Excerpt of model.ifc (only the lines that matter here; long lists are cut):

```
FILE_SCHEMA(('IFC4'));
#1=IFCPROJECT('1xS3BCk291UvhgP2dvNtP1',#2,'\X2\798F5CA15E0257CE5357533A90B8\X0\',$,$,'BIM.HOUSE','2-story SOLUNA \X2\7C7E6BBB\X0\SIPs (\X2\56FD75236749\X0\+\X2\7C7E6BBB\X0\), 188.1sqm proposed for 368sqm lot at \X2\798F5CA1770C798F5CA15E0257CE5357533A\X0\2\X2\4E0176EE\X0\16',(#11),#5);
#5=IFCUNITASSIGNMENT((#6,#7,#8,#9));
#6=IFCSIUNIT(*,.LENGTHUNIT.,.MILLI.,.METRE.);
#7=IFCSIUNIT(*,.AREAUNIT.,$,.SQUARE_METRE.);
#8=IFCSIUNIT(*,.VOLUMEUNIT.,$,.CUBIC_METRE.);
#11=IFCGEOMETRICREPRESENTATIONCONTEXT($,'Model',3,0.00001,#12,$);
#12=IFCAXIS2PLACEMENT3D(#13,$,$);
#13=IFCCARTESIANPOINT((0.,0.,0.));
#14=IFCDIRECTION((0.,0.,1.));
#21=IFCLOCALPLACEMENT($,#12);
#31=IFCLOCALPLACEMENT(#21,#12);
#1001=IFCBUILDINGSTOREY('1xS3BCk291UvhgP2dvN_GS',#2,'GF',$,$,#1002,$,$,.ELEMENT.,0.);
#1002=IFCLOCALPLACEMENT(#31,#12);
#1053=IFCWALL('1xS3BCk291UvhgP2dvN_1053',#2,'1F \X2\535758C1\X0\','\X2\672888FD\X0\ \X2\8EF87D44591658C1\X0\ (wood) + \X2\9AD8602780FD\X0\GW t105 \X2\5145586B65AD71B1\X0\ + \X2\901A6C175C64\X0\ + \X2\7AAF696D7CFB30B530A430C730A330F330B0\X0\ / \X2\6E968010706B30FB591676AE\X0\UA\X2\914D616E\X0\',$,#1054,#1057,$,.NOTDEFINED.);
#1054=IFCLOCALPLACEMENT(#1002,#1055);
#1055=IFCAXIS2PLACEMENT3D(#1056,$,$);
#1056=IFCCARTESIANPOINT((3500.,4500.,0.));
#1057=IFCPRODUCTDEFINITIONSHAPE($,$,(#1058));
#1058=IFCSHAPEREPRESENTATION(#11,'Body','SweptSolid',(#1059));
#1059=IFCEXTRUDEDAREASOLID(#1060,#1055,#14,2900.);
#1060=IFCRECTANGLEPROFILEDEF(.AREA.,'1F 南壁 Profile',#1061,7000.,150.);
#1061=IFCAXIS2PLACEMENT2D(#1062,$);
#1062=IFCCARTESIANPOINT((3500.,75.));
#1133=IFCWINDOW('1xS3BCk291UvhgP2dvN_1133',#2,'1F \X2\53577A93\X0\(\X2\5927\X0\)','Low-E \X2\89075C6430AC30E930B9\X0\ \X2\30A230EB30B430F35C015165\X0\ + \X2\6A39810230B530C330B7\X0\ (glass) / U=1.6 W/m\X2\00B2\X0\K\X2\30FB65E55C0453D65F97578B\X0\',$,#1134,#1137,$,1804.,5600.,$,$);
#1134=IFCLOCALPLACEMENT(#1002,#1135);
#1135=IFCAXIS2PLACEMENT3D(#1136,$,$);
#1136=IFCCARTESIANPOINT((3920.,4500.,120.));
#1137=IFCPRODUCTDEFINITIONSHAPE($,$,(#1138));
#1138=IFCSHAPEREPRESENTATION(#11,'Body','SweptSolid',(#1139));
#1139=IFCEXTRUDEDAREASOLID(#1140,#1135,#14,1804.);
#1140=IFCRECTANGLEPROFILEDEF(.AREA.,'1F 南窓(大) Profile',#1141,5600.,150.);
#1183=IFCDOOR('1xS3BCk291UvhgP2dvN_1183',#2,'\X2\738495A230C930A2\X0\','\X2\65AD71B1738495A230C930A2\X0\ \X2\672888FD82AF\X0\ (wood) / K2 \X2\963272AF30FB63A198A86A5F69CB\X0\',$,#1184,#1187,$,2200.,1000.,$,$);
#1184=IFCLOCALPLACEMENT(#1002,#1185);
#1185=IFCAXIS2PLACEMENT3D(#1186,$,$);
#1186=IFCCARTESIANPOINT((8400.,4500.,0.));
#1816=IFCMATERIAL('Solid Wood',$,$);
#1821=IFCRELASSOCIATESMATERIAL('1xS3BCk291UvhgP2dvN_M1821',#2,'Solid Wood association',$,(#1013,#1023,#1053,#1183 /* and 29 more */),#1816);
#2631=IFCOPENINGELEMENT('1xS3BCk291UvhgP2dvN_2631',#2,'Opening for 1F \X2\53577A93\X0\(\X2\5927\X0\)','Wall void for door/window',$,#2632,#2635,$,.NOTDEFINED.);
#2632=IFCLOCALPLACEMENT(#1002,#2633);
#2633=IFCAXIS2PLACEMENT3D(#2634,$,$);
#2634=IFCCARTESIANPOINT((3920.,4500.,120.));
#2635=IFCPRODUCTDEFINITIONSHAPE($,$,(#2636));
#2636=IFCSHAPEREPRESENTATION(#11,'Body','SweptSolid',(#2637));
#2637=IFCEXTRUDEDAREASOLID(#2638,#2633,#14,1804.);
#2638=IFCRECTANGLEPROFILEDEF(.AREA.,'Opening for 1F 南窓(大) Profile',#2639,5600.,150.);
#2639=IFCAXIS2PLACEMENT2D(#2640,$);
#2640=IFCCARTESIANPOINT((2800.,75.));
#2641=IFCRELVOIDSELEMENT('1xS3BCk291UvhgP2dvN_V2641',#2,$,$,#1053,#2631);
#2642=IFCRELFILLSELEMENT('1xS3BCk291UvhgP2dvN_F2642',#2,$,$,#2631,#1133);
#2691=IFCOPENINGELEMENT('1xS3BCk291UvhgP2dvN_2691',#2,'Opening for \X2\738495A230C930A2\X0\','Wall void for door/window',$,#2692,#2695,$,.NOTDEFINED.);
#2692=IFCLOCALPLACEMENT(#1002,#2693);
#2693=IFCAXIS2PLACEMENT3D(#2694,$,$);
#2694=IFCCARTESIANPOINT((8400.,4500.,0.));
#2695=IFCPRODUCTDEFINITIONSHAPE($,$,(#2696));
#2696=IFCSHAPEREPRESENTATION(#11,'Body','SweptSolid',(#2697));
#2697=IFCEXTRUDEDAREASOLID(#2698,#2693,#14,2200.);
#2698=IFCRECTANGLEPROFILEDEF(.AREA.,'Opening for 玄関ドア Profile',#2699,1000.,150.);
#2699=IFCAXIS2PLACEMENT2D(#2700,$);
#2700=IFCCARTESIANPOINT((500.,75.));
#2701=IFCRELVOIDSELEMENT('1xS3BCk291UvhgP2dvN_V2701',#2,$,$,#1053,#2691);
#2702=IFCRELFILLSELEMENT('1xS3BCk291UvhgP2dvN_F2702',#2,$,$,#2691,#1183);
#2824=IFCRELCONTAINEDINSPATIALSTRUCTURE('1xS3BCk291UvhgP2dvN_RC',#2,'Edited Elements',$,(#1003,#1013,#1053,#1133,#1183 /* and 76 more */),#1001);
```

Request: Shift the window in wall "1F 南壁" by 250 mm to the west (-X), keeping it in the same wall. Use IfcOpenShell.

```python
import ifcopenshell
import ifcopenshell.api.geometry
import ifcopenshell.util.placement

model = ifcopenshell.open("model.ifc")

window = model.by_id(1133)
opening = window.FillsVoids[0].RelatingOpeningElement
wall = opening.VoidsElements[0].RelatingBuildingElement

wall_matrix = ifcopenshell.util.placement.get_local_placement(wall.ObjectPlacement)
shift = wall_matrix[:3, 0] * -250.0
before = ifcopenshell.util.placement.get_local_placement(window.ObjectPlacement)[:3, 3].copy()

# The window is not placed relative to its opening, so move both.
for product in (opening, window):
    matrix = ifcopenshell.util.placement.get_local_placement(product.ObjectPlacement)
    matrix[:3, 3] += shift
    ifcopenshell.api.geometry.edit_object_placement(model, product=product, matrix=matrix, is_si=False)

after = ifcopenshell.util.placement.get_local_placement(window.ObjectPlacement)[:3, 3]
print("window moved by", (after - before).round(3) + 0.0)

model.write("model-out.ifc")
```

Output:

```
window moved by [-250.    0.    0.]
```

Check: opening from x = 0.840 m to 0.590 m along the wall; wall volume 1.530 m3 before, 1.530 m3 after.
